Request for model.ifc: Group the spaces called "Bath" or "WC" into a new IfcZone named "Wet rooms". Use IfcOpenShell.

First a look at what the model holds.

```python
import ifcopenshell

model = ifcopenshell.open("model.ifc")
print(model.schema)
seen = {}
for space in model.by_type("IfcSpace"):
    seen[space.LongName] = seen.get(space.LongName, 0) + 1
for name, count in sorted(seen.items(), key=str):
    print(count, "x", name)
print("zones:", [z.Name for z in model.by_type("IfcZone")][:20])
```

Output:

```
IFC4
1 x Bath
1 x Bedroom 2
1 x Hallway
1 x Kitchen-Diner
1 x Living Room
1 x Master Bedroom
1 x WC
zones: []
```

```python
import ifcopenshell
import ifcopenshell.api.group
import ifcopenshell.api.root

model = ifcopenshell.open("model.ifc")

names = {"Bath", "WC"}
spaces = [s for s in model.by_type("IfcSpace") if s.LongName in names]

zone = ifcopenshell.api.root.create_entity(model, ifc_class="IfcZone", name="Wet rooms")
ifcopenshell.api.group.assign_group(model, products=spaces, group=zone)
print(len(spaces), "spaces in", zone.Name)

model.write("model_edited.ifc")
```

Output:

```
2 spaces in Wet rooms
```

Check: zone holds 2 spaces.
